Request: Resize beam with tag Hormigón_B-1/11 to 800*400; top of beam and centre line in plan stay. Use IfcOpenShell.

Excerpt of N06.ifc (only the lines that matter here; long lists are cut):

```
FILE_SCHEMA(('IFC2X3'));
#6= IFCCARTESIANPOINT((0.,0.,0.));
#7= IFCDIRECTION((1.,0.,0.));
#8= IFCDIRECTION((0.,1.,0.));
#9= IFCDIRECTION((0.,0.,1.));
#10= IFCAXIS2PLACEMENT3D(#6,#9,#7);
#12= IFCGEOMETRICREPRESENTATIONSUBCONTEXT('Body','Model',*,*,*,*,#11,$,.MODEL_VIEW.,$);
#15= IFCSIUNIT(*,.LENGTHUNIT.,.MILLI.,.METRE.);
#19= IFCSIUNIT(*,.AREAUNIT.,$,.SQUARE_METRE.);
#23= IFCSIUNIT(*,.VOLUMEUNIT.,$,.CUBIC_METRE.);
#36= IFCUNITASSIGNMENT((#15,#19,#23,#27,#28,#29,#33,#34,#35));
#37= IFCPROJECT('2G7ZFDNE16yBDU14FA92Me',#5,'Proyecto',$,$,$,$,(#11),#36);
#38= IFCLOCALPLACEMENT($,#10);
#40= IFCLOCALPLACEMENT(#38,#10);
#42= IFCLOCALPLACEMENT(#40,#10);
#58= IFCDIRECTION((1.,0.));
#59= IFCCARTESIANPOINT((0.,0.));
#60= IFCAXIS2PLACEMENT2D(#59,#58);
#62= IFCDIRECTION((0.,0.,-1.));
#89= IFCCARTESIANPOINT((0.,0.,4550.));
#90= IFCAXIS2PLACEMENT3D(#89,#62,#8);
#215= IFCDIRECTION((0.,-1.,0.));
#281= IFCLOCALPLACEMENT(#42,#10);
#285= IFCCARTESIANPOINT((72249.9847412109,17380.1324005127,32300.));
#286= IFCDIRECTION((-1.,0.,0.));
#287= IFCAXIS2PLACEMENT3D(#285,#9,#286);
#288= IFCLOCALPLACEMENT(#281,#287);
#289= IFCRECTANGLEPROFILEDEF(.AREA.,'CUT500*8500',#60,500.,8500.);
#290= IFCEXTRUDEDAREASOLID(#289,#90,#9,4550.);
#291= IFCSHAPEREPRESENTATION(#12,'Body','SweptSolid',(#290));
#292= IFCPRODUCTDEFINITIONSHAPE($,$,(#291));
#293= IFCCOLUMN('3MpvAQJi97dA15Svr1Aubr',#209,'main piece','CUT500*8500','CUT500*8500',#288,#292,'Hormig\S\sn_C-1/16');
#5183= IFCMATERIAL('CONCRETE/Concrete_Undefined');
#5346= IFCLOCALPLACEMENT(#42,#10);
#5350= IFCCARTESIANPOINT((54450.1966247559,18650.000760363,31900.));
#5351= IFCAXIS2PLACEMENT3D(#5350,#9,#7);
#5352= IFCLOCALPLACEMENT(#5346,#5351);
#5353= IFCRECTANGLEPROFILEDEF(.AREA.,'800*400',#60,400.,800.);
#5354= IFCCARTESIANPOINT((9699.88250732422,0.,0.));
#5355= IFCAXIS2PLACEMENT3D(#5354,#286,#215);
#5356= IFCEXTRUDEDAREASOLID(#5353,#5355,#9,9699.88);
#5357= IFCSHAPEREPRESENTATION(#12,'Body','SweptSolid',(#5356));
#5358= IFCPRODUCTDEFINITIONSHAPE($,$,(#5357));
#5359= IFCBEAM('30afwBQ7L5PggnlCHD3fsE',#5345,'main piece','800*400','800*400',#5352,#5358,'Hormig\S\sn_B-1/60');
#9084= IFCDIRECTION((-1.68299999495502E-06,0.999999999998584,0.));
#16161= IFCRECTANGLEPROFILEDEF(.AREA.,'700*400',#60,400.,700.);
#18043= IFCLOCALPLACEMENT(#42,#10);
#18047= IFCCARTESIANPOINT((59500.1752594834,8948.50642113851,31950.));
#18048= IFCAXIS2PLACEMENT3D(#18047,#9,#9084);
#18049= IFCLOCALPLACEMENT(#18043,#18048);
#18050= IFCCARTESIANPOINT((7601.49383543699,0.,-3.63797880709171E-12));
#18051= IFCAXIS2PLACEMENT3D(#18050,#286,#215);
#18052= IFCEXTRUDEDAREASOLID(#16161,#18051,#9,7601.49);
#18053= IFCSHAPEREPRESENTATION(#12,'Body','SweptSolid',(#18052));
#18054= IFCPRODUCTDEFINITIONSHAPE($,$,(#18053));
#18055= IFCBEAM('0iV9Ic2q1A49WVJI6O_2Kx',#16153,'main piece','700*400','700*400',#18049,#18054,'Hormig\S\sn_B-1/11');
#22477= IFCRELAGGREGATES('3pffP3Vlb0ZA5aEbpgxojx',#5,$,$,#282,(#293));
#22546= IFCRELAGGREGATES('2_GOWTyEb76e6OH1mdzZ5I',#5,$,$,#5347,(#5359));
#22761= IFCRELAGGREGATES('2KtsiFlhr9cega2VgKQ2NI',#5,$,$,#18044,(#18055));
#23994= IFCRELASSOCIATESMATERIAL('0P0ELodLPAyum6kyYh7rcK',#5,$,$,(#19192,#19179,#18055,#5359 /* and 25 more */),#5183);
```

```python
import ifcopenshell
import ifcopenshell.util.element
import ifcopenshell.util.representation

model = ifcopenshell.open("N06.ifc")

member = model.by_guid("0iV9Ic2q1A49WVJI6O_2Kx")
source = next(p for p in model.by_type("IfcRectangleProfileDef") if p.ProfileName == "800*400")

body = ifcopenshell.util.representation.get_representation(member, "Model", "Body")
solid = body.Items[0]
old_profile = solid.SweptArea

# Copy the section's sizes but keep this member's own profile position.
profile = ifcopenshell.util.element.copy(model, source)
# Profiles are centred, so shift by half the change in depth to hold the top.
shift = (old_profile.YDim - profile.YDim) / 2
x, y = old_profile.Position.Location.Coordinates
up = (0.0, 1.0)  # upwards, in the solid's own plane
location = model.createIfcCartesianPoint((x + up[0] * shift, y + up[1] * shift))
profile.Position = model.createIfcAxis2Placement2D(location, old_profile.Position.RefDirection)
solid.SweptArea = profile
if not model.get_total_inverses(old_profile):
    ifcopenshell.util.element.remove_deep2(model, old_profile)
member.Description = member.Description.replace("700*400", "800*400")
member.ObjectType = member.ObjectType.replace("700*400", "800*400")

print(solid.SweptArea)

model.write("N06_rev.ifc")
```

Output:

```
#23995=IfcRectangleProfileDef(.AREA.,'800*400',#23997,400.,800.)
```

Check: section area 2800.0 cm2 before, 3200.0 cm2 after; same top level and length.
